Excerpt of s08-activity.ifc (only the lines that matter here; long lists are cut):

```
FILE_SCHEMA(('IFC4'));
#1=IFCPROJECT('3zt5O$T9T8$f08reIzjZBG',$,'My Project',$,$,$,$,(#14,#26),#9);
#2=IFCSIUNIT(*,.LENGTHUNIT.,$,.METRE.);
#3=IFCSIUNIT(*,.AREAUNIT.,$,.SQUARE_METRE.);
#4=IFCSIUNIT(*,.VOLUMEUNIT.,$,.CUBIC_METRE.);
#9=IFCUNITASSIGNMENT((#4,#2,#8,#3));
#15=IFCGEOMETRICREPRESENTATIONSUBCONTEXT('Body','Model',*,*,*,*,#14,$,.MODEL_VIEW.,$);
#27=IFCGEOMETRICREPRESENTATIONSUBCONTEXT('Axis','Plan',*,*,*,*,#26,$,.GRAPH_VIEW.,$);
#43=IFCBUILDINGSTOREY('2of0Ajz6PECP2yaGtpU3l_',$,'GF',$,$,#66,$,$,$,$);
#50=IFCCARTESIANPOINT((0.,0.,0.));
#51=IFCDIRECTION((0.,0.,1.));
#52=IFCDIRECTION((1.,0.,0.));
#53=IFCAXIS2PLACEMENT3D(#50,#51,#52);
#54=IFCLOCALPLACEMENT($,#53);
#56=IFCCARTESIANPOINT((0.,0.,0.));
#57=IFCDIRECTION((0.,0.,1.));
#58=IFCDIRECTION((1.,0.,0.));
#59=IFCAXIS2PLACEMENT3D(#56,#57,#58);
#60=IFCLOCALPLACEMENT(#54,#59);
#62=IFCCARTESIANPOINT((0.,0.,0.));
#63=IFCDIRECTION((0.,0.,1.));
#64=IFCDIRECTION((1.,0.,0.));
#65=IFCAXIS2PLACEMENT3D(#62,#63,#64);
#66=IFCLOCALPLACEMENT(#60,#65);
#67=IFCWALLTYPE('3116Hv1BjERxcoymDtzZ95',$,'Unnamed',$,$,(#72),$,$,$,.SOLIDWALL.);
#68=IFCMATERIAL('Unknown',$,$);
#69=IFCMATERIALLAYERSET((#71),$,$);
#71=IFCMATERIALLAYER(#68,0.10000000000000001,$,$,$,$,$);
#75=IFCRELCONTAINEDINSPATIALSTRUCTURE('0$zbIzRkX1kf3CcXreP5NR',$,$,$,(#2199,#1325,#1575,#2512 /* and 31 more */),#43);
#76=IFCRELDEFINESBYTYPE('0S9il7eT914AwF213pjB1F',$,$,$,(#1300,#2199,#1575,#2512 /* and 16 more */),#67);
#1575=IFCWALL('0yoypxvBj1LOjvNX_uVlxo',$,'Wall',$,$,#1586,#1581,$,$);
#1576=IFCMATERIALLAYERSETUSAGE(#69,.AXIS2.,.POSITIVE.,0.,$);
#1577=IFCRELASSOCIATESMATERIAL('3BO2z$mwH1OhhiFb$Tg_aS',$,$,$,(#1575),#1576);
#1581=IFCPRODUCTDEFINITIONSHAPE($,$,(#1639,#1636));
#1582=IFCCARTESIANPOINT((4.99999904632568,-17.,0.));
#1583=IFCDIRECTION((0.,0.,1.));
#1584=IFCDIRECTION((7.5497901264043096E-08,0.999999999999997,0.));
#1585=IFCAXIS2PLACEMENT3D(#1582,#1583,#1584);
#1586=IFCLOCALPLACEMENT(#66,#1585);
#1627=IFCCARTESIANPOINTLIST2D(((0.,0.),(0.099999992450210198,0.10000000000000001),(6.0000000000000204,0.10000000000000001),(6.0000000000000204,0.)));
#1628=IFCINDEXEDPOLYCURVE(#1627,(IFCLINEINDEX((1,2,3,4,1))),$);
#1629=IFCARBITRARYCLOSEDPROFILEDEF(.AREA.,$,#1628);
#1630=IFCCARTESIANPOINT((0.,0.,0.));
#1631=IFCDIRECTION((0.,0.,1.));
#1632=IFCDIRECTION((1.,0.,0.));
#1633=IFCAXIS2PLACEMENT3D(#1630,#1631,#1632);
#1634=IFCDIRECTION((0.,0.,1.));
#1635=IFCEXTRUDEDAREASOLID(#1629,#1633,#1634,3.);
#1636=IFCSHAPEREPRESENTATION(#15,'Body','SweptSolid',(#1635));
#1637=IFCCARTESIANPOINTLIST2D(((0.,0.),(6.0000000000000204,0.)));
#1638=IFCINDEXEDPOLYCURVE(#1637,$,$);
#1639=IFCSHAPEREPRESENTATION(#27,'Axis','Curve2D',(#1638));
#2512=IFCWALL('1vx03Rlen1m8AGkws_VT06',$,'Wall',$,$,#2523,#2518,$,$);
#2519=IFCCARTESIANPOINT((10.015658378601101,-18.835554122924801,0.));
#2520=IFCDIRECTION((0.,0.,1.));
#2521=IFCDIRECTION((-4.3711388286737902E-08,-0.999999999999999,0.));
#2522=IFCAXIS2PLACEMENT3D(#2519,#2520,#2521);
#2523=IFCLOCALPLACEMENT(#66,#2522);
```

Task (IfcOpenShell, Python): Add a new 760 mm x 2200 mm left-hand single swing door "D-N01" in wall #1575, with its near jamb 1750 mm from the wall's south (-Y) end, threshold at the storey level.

```python
import numpy as np
import ifcopenshell
import ifcopenshell.api.feature
import ifcopenshell.api.geometry
import ifcopenshell.api.root
import ifcopenshell.api.spatial
import ifcopenshell.geom
import ifcopenshell.util.element
import ifcopenshell.util.placement
import ifcopenshell.util.representation
import ifcopenshell.util.shape
import ifcopenshell.util.unit

model = ifcopenshell.open("s08-activity.ifc")
unit_scale = ifcopenshell.util.unit.calculate_unit_scale(model)
settings = ifcopenshell.geom.settings()


def volume(element):
    """Net volume in cubic metres, openings subtracted."""
    shape = ifcopenshell.geom.create_shape(settings, element)
    return ifcopenshell.util.shape.get_volume(shape.geometry)


wall = model.by_id(1575)
storey = ifcopenshell.util.element.get_container(wall, ifc_class="IfcBuildingStorey")
context = ifcopenshell.util.representation.get_context(model, "Model", "Body", "MODEL_VIEW")
before = volume(wall)

width, height, from_end, sill = 0.76, 2.2, 1.75, 0.0  # metres

# The wall runs along its own X axis, and the end named is its -X end.
wall_shape = ifcopenshell.geom.create_shape(settings, wall)
x, y, z = ifcopenshell.util.shape.get_vertices(wall_shape.geometry).T
start = x.min() + from_end
face, thickness = float(y.min()), float(y.max() - y.min())
wall_matrix = ifcopenshell.util.placement.get_local_placement(wall.ObjectPlacement)
level = ifcopenshell.util.placement.get_local_placement(storey.ObjectPlacement)[2, 3]


def in_wall(x, y):
    """Placement at x, y metres in the wall's axes, at sill height."""
    matrix = wall_matrix.copy()
    matrix[:, 3] = wall_matrix @ np.array([x / unit_scale, y / unit_scale, 0.0, 1.0])
    matrix[2, 3] = level + sill / unit_scale
    return matrix


# Opening: a box that overshoots both wall faces by 50 mm.
opening = ifcopenshell.api.root.create_entity(model, ifc_class="IfcOpeningElement", predefined_type="OPENING")
box = ifcopenshell.api.geometry.add_wall_representation(
    model, context=context, length=width, height=height, thickness=thickness + 0.1
)
ifcopenshell.api.geometry.assign_representation(model, product=opening, representation=box)
ifcopenshell.api.geometry.edit_object_placement(model, product=opening, matrix=in_wall(start, face - 0.05), is_si=False)
ifcopenshell.api.feature.add_feature(model, feature=opening, element=wall)

door = ifcopenshell.api.root.create_entity(model, ifc_class="IfcDoor", name="D-N01", predefined_type="DOOR")
door.OverallWidth, door.OverallHeight = width / unit_scale, height / unit_scale
door.OperationType = "SINGLE_SWING_LEFT"
body = ifcopenshell.api.geometry.add_door_representation(
    model,
    context=context,
    overall_width=door.OverallWidth,
    overall_height=door.OverallHeight,
    operation_type="SINGLE_SWING_LEFT",
    lining_properties={"LiningDepth": thickness / unit_scale, "ThresholdDepth": thickness / unit_scale},
)
ifcopenshell.api.geometry.assign_representation(model, product=door, representation=body)
ifcopenshell.api.spatial.assign_container(model, products=[door], relating_structure=storey)
ifcopenshell.api.feature.add_filling(model, opening=opening, element=door)

# The lining spans the wall, so the door starts at the wall face.
ifcopenshell.api.geometry.edit_object_placement(model, product=door, matrix=in_wall(start, face), is_si=False)

after = volume(wall)

print(f"wall volume {before:.3f} -> {after:.3f} m3")

model.write("s08-activity_v2.ifc")
```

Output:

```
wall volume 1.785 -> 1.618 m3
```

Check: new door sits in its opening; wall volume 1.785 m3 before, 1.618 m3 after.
